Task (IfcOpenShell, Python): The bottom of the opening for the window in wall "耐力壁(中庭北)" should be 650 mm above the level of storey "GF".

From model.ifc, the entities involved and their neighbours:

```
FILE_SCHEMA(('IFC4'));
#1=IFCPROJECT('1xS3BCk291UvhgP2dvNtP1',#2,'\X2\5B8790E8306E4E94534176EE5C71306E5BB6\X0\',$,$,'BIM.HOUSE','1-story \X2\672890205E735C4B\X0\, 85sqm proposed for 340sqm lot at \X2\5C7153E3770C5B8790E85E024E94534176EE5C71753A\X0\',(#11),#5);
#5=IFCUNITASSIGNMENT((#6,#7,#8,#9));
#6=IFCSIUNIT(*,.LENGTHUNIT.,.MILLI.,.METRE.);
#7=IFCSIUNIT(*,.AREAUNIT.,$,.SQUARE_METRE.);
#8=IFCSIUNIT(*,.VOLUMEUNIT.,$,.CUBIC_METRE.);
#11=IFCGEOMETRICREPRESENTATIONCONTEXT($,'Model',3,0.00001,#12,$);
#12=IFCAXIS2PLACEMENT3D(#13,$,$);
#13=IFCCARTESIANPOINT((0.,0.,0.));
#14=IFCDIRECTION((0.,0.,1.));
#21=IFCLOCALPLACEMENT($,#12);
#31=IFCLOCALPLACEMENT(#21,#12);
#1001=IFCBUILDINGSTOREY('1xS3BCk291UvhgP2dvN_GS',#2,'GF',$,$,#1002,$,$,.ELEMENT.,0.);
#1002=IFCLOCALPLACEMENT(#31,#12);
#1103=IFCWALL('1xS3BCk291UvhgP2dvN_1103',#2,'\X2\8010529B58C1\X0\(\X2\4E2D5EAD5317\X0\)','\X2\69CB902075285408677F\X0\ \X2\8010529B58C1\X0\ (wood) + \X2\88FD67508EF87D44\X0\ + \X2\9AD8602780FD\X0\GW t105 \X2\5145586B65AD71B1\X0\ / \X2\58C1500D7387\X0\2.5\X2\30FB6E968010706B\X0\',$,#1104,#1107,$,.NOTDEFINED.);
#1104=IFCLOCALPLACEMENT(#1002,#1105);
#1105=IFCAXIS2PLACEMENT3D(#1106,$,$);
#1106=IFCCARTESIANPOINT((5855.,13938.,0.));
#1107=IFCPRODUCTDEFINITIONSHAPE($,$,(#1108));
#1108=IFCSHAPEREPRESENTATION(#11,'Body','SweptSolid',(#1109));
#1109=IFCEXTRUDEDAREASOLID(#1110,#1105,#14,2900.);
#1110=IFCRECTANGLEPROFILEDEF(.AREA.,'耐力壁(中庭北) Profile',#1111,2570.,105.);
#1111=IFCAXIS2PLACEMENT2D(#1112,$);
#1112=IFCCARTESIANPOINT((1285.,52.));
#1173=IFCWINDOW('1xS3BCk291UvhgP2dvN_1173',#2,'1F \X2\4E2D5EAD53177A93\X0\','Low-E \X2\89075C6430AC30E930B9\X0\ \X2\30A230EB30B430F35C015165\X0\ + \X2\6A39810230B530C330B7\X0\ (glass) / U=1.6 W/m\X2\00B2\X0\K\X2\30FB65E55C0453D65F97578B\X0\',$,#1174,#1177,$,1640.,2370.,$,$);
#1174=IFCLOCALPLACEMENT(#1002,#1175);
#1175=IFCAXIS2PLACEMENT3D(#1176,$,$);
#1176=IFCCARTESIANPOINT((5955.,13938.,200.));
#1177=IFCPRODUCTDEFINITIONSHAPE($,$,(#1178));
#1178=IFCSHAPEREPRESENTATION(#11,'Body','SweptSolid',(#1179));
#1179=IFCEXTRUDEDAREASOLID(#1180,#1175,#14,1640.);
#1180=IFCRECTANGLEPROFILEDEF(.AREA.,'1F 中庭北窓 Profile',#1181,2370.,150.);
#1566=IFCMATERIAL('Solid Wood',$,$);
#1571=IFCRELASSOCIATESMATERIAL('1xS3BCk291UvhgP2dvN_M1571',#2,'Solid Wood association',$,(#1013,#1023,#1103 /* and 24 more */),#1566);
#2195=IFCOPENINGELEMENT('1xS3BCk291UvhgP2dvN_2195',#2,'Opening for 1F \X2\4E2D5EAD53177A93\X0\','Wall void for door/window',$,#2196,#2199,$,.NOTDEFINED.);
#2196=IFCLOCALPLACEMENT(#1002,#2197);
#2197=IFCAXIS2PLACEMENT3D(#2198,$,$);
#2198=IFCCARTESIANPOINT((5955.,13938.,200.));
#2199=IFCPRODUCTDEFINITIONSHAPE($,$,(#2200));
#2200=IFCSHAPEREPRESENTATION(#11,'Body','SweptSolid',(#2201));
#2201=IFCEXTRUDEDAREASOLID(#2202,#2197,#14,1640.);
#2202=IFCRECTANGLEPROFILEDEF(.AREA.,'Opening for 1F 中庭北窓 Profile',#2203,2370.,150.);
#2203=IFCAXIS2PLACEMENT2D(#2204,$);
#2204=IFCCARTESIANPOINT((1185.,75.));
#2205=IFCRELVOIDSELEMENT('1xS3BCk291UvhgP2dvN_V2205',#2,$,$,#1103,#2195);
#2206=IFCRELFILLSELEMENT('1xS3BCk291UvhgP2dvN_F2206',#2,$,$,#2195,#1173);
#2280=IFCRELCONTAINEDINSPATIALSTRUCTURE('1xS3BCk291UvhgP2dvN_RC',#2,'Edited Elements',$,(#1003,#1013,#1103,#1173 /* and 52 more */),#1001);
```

```python
import numpy as np
import ifcopenshell
import ifcopenshell.api.geometry
import ifcopenshell.geom
import ifcopenshell.util.element
import ifcopenshell.util.placement
import ifcopenshell.util.shape
import ifcopenshell.util.unit

model = ifcopenshell.open("model.ifc")
unit_scale = ifcopenshell.util.unit.calculate_unit_scale(model)

window = model.by_guid("1xS3BCk291UvhgP2dvN_1173")
opening = window.FillsVoids[0].RelatingOpeningElement
storey = ifcopenshell.util.element.get_container(window, ifc_class="IfcBuildingStorey")
level = ifcopenshell.util.placement.get_local_placement(storey.ObjectPlacement)[2, 3]

# The opening's origin need not be at the sill, so measure its lowest point.
shape = ifcopenshell.geom.create_shape(ifcopenshell.geom.settings(), opening)
bottom = ifcopenshell.util.shape.get_shape_bottom_elevation(shape, shape.geometry) / unit_scale
dz = level + 0.65 / unit_scale - bottom

shift = np.array([0.0, 0.0, dz])
# The window is not placed relative to its opening, so move both.
for product in (opening, window):
    matrix = ifcopenshell.util.placement.get_local_placement(product.ObjectPlacement)
    matrix[:3, 3] += shift
    ifcopenshell.api.geometry.edit_object_placement(model, product=product, matrix=matrix, is_si=False)

print(f"moved by {dz * unit_scale:+.3f} m")

model.write("model_edited.ifc")
```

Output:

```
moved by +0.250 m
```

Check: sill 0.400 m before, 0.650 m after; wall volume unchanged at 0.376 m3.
